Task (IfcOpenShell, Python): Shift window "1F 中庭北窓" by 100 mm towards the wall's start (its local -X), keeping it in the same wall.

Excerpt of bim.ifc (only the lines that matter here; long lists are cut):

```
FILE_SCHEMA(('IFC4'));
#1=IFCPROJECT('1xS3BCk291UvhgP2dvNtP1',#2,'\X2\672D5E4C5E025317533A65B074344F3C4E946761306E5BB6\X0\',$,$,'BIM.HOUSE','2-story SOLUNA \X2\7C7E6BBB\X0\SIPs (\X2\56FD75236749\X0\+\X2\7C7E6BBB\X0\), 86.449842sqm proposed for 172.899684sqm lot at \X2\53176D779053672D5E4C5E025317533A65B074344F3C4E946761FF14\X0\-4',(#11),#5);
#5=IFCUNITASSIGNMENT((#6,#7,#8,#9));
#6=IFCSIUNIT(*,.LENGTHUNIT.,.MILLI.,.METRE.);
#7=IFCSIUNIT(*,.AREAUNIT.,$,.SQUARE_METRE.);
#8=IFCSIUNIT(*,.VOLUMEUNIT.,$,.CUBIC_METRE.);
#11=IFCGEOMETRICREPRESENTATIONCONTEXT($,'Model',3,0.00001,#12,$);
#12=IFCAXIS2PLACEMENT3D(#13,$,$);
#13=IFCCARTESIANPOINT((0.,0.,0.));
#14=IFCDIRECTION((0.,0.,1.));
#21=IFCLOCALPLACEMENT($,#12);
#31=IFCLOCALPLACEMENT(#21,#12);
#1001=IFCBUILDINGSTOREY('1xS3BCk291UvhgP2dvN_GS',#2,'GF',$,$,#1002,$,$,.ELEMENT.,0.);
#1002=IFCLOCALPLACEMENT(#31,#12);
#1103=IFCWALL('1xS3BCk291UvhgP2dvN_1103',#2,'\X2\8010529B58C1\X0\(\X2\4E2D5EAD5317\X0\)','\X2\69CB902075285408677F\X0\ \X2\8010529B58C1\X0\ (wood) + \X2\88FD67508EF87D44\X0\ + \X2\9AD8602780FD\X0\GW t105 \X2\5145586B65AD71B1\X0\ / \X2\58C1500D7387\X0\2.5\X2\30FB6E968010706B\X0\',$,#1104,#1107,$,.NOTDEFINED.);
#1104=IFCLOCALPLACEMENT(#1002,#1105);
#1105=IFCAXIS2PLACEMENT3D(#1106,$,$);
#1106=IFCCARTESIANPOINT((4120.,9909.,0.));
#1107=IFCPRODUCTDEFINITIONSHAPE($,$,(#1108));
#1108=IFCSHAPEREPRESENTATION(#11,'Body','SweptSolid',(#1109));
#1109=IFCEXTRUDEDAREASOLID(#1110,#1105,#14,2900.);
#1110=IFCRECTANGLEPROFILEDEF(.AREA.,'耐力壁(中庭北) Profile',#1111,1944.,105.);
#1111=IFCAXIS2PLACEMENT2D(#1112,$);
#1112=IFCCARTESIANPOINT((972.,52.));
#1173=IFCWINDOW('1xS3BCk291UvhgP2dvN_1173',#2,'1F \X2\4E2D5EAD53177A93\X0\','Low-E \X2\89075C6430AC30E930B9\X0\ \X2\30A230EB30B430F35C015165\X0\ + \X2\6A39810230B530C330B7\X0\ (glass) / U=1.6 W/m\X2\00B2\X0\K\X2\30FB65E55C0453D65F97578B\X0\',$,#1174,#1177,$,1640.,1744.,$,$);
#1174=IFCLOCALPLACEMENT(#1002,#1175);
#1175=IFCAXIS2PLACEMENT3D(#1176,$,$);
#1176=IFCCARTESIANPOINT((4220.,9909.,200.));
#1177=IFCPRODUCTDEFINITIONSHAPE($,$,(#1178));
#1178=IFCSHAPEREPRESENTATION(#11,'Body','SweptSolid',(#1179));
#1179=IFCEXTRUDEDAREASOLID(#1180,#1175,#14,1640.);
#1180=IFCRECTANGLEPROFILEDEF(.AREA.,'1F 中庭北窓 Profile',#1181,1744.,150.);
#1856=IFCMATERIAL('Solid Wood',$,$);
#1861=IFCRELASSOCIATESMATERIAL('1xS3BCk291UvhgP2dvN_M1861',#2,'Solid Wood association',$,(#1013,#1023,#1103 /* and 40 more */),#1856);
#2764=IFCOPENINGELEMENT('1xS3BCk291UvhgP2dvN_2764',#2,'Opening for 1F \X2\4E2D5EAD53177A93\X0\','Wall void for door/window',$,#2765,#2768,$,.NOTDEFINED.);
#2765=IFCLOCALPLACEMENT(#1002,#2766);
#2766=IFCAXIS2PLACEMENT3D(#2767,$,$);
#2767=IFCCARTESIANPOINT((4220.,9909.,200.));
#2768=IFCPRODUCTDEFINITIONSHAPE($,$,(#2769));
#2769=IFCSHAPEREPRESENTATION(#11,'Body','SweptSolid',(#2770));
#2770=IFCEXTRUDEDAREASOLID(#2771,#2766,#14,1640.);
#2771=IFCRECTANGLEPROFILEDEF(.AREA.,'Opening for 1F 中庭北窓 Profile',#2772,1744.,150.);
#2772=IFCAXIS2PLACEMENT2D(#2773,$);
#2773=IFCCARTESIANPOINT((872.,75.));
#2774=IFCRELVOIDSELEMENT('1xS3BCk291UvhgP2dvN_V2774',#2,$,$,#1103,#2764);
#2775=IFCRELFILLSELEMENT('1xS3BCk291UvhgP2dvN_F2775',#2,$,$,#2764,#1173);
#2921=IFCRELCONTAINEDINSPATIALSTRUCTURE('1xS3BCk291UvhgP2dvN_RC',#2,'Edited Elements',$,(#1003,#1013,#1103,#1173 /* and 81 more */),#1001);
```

```python
import ifcopenshell
import ifcopenshell.api.geometry
import ifcopenshell.util.placement
import ifcopenshell.util.unit

model = ifcopenshell.open("bim.ifc")
unit_scale = ifcopenshell.util.unit.calculate_unit_scale(model)

window = model.by_guid("1xS3BCk291UvhgP2dvN_1173")
opening = window.FillsVoids[0].RelatingOpeningElement
wall = opening.VoidsElements[0].RelatingBuildingElement

wall_matrix = ifcopenshell.util.placement.get_local_placement(wall.ObjectPlacement)
shift = wall_matrix[:3, 0] * -0.1 / unit_scale
before = ifcopenshell.util.placement.get_local_placement(window.ObjectPlacement)[:3, 3].copy()

# The window is not placed relative to its opening, so move both.
for product in (opening, window):
    matrix = ifcopenshell.util.placement.get_local_placement(product.ObjectPlacement)
    matrix[:3, 3] += shift
    ifcopenshell.api.geometry.edit_object_placement(model, product=product, matrix=matrix, is_si=False)

after = ifcopenshell.util.placement.get_local_placement(window.ObjectPlacement)[:3, 3]
print("window moved by", (after - before).round(3) + 0.0)

model.write("bim_v2.ifc")
```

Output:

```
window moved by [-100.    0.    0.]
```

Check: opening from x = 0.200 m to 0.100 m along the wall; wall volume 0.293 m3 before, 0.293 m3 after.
